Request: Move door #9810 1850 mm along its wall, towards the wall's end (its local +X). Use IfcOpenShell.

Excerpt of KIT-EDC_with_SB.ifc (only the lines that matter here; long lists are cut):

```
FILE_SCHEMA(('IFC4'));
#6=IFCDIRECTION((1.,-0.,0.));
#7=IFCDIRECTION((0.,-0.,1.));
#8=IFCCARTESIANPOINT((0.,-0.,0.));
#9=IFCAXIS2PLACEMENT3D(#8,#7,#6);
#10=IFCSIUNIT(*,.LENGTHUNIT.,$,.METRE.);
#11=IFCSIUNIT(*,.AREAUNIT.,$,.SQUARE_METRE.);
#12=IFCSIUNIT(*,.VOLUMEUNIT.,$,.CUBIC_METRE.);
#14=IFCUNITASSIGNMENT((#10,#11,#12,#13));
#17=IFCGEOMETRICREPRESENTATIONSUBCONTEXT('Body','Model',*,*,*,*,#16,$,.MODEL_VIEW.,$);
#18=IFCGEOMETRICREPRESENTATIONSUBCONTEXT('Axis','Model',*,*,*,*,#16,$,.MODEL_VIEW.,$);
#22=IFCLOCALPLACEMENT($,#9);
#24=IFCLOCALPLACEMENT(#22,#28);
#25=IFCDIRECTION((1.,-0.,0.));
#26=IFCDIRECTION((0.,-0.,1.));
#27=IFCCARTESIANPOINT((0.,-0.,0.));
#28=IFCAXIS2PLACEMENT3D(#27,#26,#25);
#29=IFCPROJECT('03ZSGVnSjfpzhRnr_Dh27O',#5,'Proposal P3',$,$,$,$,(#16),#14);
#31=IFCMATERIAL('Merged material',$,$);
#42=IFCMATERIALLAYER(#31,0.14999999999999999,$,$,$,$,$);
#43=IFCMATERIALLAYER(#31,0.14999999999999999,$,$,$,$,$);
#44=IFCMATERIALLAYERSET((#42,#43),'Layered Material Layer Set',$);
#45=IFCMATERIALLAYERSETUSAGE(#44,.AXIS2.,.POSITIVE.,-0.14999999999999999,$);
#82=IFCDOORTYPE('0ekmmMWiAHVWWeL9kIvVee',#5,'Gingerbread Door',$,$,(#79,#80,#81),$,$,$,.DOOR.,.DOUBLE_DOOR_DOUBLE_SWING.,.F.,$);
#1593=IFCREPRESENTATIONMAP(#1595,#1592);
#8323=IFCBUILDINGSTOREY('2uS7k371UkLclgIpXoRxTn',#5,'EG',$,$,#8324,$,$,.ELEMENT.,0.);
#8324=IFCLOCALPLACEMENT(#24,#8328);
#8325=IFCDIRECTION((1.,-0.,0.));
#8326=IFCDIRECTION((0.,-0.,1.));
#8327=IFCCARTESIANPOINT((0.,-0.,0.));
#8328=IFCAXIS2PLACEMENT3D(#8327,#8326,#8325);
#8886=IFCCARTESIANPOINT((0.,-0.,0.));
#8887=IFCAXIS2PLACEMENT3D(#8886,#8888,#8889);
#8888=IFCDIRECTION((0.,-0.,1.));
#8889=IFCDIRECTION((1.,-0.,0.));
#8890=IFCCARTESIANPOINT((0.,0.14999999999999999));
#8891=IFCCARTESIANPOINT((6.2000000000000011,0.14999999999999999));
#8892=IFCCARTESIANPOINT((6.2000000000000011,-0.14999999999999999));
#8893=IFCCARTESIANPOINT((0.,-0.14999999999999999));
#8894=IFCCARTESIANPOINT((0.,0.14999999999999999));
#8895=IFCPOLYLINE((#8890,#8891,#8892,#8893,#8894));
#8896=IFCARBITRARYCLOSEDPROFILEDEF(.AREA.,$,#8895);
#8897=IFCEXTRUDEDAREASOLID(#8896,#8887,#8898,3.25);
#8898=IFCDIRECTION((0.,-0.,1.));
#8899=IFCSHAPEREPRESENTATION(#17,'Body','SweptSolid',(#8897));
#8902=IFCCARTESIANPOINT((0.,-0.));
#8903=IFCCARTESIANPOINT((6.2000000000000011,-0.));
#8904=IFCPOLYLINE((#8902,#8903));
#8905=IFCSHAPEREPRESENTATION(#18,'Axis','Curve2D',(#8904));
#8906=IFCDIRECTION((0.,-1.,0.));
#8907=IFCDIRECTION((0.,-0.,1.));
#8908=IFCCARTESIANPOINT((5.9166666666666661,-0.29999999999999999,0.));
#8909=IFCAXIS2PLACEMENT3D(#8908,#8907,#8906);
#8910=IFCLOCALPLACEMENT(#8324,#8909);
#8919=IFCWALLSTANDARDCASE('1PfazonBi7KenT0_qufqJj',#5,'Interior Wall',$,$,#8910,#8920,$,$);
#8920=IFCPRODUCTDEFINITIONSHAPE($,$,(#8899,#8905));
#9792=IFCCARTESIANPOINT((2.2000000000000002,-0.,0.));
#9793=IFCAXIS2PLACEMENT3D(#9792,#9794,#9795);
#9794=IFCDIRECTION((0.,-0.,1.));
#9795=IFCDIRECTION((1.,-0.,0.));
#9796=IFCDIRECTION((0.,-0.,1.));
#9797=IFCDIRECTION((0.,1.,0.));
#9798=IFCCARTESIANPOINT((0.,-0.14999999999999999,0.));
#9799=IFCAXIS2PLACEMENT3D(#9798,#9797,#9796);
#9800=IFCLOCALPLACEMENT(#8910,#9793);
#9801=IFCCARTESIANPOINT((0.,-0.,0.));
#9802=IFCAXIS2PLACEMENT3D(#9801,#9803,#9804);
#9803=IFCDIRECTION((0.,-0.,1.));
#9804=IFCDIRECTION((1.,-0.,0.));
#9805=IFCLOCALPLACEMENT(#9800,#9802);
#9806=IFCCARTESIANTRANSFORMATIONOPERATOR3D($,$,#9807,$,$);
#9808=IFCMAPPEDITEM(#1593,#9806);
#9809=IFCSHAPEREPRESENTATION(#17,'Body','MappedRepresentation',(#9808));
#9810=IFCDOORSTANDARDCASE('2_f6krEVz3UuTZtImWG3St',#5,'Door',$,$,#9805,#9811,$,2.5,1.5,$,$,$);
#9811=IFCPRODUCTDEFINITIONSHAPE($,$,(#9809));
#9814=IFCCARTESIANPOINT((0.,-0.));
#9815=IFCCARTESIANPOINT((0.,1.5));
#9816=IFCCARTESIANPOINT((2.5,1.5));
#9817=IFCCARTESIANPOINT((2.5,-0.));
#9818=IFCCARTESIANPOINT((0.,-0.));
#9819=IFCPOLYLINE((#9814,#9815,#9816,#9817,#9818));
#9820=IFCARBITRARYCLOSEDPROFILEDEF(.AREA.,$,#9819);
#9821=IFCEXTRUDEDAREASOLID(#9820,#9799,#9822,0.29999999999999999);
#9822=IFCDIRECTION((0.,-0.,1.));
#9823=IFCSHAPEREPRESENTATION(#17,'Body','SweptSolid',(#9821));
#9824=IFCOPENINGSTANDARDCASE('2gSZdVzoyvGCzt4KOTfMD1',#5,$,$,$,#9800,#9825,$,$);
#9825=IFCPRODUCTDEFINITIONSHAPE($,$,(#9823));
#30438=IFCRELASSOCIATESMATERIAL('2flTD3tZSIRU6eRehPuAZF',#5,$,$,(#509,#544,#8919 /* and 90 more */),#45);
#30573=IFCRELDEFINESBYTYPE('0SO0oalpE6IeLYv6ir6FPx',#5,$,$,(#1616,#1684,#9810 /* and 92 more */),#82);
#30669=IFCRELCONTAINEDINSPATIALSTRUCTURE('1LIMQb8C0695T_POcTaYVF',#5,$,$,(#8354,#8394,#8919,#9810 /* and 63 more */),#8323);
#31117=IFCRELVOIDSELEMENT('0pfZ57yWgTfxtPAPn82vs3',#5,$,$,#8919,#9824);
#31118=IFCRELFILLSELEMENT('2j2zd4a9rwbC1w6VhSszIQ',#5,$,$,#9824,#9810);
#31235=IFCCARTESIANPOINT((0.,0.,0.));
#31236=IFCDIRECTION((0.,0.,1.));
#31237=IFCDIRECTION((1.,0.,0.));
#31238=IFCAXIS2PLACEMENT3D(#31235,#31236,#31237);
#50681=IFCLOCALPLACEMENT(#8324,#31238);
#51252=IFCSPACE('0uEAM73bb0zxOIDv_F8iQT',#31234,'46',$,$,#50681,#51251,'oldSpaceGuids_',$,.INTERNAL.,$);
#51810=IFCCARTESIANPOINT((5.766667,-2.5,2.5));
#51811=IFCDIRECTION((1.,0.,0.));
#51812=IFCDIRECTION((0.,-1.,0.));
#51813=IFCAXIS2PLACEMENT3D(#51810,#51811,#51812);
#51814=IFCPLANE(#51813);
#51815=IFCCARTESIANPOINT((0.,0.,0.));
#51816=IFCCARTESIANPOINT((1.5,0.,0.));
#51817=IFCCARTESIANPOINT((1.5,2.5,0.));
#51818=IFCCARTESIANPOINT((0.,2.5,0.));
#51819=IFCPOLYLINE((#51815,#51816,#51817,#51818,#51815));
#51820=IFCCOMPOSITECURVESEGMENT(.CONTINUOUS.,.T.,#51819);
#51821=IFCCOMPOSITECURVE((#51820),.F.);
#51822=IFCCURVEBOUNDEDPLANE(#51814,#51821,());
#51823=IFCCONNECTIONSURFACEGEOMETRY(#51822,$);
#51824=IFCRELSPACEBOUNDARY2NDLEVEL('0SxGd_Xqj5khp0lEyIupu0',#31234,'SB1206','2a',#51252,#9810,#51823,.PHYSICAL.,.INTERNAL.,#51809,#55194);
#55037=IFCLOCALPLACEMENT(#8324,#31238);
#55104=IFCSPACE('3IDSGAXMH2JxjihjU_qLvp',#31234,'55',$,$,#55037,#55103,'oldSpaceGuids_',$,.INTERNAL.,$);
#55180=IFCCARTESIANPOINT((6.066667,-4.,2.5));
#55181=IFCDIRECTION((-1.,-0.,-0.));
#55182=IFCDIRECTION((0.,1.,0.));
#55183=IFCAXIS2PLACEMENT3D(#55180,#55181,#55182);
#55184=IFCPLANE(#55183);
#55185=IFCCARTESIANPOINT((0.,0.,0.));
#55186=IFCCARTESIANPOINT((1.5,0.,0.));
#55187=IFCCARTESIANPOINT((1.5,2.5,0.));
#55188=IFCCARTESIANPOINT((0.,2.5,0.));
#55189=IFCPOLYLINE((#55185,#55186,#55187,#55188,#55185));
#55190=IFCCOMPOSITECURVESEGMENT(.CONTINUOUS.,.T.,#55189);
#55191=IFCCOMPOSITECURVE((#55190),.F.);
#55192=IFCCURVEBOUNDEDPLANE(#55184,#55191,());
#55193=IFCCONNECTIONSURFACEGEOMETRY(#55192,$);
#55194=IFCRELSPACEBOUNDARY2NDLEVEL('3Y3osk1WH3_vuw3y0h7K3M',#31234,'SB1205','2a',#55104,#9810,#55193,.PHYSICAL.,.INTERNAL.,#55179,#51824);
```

```python
import numpy as np
import ifcopenshell
import ifcopenshell.api.geometry
import ifcopenshell.util.placement
import ifcopenshell.util.unit

model = ifcopenshell.open("KIT-EDC_with_SB.ifc")
unit_scale = ifcopenshell.util.unit.calculate_unit_scale(model)

door = model.by_guid("2_f6krEVz3UuTZtImWG3St")
opening = door.FillsVoids[0].RelatingOpeningElement
wall = opening.VoidsElements[0].RelatingBuildingElement

wall_matrix = ifcopenshell.util.placement.get_local_placement(wall.ObjectPlacement)
shift = wall_matrix[:3, 0] * 1.85 / unit_scale
before = ifcopenshell.util.placement.get_local_placement(door.ObjectPlacement)[:3, 3].copy()

# The door is placed relative to its opening, so it follows when the opening moves.
matrix = ifcopenshell.util.placement.get_local_placement(opening.ObjectPlacement)
matrix[:3, 3] += shift
ifcopenshell.api.geometry.edit_object_placement(
    model, product=opening, matrix=matrix, is_si=False, should_transform_children=True
)

# Space boundary surfaces are stored in each space's coordinates; move them too.
for rel in door.ProvidesBoundaries:
    if not rel.ConnectionGeometry:
        continue
    surface = rel.ConnectionGeometry.SurfaceOnRelatingElement.BasisSurface
    space_matrix = ifcopenshell.util.placement.get_local_placement(rel.RelatingSpace.ObjectPlacement)
    point = np.array(surface.Position.Location.Coordinates) + space_matrix[:3, :3].T @ shift
    surface.Position = model.createIfcAxis2Placement3D(
        model.createIfcCartesianPoint(point.tolist()), surface.Position.Axis, surface.Position.RefDirection
    )

after = ifcopenshell.util.placement.get_local_placement(door.ObjectPlacement)[:3, 3]
print("door moved by", (after - before).round(3) + 0.0)

model.write("KIT-EDC_with_SB_rev.ifc")
```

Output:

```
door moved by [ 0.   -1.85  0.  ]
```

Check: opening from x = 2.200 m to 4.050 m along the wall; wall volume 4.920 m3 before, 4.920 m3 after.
